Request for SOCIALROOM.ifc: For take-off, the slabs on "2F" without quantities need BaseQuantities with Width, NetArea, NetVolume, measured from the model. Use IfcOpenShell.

First a look at what the model holds.

```python
import ifcopenshell
import ifcopenshell.util.element
import ifcopenshell.util.unit

model = ifcopenshell.open("SOCIALROOM.ifc")
print(model.schema)
for unit_type in ("LENGTHUNIT", "AREAUNIT", "VOLUMEUNIT"):
    print(unit_type, ifcopenshell.util.unit.calculate_unit_scale(model, unit_type))
storey = next(s for s in model.by_type("IfcBuildingStorey") if s.Name == "2F")
slabs = [e for e in ifcopenshell.util.element.get_decomposition(storey) if e.is_a("IfcSlab")]
for e in sorted(slabs, key=lambda e: e.id()):
    print(e.id(), e.is_a(), e.Name, list(ifcopenshell.util.element.get_psets(e, qtos_only=True)), sep=" | ")
```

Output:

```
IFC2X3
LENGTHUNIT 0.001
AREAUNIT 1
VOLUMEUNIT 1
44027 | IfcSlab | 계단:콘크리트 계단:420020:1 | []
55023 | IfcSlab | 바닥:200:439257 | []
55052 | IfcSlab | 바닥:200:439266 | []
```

```python
import ifcopenshell
import ifcopenshell.api.pset
import ifcopenshell.geom
import ifcopenshell.util.element
import ifcopenshell.util.shape
import ifcopenshell.util.unit

model = ifcopenshell.open("SOCIALROOM.ifc")
unit_scale = ifcopenshell.util.unit.calculate_unit_scale(model)
area_scale = ifcopenshell.util.unit.calculate_unit_scale(model, "AREAUNIT")
volume_scale = ifcopenshell.util.unit.calculate_unit_scale(model, "VOLUMEUNIT")
settings = ifcopenshell.geom.settings()

storey = next(s for s in model.by_type("IfcBuildingStorey") if s.Name == "2F")
slabs = [e for e in ifcopenshell.util.element.get_decomposition(storey) if e.is_a("IfcSlab")]

for e in sorted(slabs, key=lambda e: e.id()):
    if ifcopenshell.util.element.get_psets(e, qtos_only=True, should_inherit=False):
        continue
    # Geometry comes back in metres, in the element's own axes.
    shape = ifcopenshell.geom.create_shape(settings, e)
    values = {
        "Width": ifcopenshell.util.shape.get_z(shape.geometry) / unit_scale,
        "NetArea": ifcopenshell.util.shape.get_footprint_area(shape.geometry) / area_scale,
        "NetVolume": ifcopenshell.util.shape.get_volume(shape.geometry) / volume_scale,
    }
    qto = ifcopenshell.api.pset.add_qto(model, product=e, name="BaseQuantities")
    ifcopenshell.api.pset.edit_qto(model, qto=qto, properties=values)
    print(e.id(), {k: round(v, 3) for k, v in values.items()})

model.write("SOCIALROOM_updated.ifc")
```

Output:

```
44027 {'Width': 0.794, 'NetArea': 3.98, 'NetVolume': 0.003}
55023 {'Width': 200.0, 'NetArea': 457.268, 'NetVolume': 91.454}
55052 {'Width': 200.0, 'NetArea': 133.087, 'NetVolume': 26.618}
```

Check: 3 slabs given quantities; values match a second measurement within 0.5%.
